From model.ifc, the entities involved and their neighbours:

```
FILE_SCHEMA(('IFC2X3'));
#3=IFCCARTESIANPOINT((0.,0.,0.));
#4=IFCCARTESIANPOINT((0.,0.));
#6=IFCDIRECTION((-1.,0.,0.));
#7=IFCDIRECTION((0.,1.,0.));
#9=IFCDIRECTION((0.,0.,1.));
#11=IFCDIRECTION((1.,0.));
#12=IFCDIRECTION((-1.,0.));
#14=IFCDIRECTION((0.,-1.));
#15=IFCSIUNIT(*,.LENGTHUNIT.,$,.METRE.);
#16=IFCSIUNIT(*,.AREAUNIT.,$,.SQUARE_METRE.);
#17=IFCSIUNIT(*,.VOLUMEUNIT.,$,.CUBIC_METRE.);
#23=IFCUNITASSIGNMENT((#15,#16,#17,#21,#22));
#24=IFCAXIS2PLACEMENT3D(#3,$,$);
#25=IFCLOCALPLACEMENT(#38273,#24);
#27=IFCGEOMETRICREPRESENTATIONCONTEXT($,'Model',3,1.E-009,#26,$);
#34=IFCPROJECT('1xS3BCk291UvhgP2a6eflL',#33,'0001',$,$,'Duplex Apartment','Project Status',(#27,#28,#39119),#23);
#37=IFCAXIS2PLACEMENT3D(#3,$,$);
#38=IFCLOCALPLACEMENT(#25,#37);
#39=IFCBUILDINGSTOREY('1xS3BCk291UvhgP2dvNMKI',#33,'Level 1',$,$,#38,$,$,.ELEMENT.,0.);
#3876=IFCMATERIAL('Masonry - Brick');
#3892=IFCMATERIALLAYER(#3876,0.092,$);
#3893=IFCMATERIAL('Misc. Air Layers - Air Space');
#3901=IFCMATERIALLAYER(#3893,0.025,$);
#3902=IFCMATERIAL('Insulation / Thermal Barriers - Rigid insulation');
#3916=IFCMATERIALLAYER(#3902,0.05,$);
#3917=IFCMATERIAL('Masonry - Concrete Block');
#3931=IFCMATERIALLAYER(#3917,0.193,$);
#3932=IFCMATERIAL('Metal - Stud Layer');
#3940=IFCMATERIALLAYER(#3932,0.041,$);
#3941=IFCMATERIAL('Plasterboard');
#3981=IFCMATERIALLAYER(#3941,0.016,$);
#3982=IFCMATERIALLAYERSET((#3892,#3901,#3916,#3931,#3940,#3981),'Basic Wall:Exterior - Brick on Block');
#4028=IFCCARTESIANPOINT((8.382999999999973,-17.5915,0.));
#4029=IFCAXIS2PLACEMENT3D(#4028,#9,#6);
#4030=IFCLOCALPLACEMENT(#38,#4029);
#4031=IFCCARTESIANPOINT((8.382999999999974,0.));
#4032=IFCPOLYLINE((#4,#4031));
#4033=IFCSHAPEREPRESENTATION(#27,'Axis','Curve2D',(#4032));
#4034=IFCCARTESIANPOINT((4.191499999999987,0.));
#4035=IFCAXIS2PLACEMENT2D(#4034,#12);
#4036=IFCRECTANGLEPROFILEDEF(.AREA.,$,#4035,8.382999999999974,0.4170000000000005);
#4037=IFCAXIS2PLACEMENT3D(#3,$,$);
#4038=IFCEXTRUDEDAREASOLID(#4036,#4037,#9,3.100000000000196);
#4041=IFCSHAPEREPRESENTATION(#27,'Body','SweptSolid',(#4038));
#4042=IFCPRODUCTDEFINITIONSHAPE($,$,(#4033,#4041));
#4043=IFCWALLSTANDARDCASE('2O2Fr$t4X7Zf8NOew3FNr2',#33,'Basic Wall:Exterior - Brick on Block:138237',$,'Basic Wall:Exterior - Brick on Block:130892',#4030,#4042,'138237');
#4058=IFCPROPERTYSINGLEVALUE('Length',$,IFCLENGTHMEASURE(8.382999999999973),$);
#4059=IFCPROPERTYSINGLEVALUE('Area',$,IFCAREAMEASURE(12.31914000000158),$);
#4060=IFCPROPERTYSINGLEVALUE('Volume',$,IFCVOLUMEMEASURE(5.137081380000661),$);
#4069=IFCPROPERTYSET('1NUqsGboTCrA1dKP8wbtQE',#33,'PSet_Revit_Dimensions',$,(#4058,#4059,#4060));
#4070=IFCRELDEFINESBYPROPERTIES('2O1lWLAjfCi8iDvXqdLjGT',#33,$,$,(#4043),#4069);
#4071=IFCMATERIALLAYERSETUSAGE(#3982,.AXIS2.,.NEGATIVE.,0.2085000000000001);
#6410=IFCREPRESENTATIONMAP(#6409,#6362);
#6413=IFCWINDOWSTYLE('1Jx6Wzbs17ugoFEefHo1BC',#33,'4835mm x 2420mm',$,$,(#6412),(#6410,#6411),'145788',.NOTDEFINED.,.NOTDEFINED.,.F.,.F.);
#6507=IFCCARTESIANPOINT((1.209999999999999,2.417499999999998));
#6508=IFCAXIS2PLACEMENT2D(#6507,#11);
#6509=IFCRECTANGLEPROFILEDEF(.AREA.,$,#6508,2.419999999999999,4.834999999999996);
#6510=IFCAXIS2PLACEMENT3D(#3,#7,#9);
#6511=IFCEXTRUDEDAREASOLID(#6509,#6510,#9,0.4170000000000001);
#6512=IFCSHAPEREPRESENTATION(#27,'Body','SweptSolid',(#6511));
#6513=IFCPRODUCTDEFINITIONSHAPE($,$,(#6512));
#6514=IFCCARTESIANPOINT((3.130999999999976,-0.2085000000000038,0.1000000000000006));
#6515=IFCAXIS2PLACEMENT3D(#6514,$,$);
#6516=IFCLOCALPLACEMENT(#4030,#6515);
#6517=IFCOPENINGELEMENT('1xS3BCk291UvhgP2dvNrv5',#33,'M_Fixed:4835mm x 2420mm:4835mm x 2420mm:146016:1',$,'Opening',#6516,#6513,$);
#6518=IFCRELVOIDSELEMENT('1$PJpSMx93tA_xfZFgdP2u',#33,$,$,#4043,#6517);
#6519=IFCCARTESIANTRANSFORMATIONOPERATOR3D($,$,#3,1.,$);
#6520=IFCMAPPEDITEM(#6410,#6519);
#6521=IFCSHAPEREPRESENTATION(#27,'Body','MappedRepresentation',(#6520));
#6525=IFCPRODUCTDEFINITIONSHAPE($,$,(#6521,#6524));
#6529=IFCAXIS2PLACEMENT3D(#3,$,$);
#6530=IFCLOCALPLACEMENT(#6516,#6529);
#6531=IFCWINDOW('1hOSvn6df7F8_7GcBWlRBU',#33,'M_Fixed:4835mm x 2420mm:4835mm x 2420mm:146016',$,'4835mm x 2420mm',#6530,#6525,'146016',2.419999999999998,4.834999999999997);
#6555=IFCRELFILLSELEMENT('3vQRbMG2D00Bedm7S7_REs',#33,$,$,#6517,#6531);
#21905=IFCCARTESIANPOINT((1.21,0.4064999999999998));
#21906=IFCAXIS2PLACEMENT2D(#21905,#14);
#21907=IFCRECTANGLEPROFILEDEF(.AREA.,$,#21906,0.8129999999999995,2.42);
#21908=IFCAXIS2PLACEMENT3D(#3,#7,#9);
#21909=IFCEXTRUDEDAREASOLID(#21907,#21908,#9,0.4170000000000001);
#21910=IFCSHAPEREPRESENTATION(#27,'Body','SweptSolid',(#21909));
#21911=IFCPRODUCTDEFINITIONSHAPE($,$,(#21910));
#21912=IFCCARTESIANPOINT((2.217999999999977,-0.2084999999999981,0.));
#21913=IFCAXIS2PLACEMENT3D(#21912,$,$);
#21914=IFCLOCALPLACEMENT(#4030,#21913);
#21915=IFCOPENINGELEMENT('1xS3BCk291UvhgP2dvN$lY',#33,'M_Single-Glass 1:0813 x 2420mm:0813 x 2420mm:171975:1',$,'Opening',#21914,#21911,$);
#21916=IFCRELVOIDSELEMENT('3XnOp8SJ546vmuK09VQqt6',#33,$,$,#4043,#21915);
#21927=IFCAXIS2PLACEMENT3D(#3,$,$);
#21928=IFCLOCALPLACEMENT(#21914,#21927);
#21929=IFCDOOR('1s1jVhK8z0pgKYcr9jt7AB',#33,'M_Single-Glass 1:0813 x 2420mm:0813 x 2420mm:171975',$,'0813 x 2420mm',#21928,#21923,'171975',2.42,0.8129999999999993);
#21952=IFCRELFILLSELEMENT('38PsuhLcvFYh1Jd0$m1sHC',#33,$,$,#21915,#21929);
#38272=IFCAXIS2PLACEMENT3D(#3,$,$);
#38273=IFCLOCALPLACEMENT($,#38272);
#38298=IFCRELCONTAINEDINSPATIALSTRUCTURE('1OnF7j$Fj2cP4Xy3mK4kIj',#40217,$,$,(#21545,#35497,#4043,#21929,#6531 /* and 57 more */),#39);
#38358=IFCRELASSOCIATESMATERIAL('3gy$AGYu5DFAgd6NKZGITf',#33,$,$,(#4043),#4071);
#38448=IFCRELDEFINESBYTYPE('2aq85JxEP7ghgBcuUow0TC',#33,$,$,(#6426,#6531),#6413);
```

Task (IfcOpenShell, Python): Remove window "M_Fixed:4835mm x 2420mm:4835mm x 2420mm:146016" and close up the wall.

```python
import ifcopenshell
import ifcopenshell.api.feature
import ifcopenshell.api.pset
import ifcopenshell.api.root
import ifcopenshell.geom
import ifcopenshell.util.element
import ifcopenshell.util.shape
import ifcopenshell.util.unit

model = ifcopenshell.open("model.ifc")
area_scale = ifcopenshell.util.unit.calculate_unit_scale(model, "AREAUNIT")
volume_scale = ifcopenshell.util.unit.calculate_unit_scale(model, "VOLUMEUNIT")
settings = ifcopenshell.geom.settings()


def volume(element):
    """Net volume in cubic metres, openings subtracted."""
    shape = ifcopenshell.geom.create_shape(settings, element)
    return ifcopenshell.util.shape.get_volume(shape.geometry)


window = model.by_id(6531)
opening = window.FillsVoids[0].RelatingOpeningElement
wall = opening.VoidsElements[0].RelatingBuildingElement
before = volume(wall)

ifcopenshell.api.root.remove_product(model, product=window)
ifcopenshell.api.feature.remove_feature(model, feature=opening)

after = volume(wall)
thickness = 0.417  # wall thickness in metres

# Update the wall's stored quantities.
pset = model.by_id(ifcopenshell.util.element.get_pset(wall, "PSet_Revit_Dimensions", should_inherit=False)["id"])
ifcopenshell.api.pset.edit_pset(model, pset=pset, properties={
    "Area": model.create_entity("IfcAreaMeasure", after / thickness / area_scale),
    "Volume": model.create_entity("IfcVolumeMeasure", after / volume_scale),
})

print(f"wall volume {before:.3f} -> {after:.3f} m3")

model.write("model_v2.ifc")
```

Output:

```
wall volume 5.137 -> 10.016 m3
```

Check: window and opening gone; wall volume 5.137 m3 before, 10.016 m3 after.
